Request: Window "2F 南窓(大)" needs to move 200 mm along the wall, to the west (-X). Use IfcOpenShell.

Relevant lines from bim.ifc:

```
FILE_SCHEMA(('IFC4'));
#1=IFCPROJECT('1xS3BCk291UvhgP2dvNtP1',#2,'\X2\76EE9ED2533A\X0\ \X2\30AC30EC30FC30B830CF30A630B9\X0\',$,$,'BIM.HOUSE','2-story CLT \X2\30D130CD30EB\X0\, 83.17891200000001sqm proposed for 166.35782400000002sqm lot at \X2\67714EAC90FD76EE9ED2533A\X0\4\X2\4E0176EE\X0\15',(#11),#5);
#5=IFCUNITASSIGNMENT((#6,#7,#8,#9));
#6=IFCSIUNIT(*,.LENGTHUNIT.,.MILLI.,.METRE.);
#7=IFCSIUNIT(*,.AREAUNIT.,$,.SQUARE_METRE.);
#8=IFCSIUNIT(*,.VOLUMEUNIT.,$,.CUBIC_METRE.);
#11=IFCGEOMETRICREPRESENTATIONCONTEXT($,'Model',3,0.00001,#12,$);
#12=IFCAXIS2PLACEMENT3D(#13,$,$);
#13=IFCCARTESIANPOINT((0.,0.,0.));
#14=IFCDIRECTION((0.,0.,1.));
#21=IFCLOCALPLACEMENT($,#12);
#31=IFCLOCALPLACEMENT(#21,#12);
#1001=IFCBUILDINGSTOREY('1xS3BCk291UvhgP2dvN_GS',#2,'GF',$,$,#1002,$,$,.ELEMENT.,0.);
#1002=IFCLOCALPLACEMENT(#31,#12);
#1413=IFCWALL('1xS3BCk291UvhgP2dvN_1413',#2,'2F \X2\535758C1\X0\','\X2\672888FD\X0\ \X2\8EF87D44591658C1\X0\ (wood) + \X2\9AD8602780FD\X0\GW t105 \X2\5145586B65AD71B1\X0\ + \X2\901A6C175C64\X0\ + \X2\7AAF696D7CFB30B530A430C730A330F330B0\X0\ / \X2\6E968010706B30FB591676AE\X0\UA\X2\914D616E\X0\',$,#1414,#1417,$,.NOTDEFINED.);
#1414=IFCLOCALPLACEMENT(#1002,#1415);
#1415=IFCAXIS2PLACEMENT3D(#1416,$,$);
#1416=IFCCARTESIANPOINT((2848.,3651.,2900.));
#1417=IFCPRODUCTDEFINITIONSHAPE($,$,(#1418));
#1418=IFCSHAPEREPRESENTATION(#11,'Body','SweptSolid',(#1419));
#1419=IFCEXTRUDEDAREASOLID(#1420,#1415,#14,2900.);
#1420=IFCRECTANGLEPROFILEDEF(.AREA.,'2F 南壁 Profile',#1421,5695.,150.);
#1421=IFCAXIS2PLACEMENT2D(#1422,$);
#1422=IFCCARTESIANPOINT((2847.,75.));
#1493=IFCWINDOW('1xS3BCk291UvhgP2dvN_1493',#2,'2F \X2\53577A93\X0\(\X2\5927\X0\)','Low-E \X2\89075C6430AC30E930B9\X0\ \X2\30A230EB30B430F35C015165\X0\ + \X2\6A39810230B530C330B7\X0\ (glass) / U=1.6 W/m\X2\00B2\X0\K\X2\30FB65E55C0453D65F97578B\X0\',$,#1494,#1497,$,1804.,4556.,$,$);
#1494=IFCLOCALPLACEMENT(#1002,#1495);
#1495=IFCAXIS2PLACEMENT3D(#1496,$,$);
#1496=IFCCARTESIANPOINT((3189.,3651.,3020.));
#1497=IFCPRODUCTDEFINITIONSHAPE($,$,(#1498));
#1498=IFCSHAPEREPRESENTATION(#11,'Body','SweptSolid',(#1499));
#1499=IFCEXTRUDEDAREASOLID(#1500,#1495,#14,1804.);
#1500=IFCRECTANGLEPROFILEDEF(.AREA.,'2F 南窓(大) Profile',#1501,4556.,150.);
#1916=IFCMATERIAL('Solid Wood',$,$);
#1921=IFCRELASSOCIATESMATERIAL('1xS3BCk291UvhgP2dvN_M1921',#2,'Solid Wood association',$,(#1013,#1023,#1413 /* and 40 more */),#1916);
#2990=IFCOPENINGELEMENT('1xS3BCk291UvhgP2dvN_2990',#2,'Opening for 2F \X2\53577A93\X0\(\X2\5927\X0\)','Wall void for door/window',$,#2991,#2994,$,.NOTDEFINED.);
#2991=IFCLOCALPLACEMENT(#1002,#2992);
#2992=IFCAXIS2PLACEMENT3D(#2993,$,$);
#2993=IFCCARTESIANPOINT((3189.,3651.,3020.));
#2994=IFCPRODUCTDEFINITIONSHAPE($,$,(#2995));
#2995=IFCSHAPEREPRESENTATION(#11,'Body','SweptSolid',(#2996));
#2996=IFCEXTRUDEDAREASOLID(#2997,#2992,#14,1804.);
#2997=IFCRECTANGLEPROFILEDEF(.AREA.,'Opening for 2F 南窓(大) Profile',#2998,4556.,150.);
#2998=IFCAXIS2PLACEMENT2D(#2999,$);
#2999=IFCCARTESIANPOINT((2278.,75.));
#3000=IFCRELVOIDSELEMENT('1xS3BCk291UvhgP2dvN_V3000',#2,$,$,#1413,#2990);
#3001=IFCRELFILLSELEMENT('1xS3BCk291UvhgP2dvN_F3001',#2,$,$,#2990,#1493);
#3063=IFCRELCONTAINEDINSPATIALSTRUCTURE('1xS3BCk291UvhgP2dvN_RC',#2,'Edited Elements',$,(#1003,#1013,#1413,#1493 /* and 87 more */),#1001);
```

```python
import ifcopenshell
import ifcopenshell.api.geometry
import ifcopenshell.util.placement
import ifcopenshell.util.unit

model = ifcopenshell.open("bim.ifc")
unit_scale = ifcopenshell.util.unit.calculate_unit_scale(model)

window = model.by_guid("1xS3BCk291UvhgP2dvN_1493")
opening = window.FillsVoids[0].RelatingOpeningElement
wall = opening.VoidsElements[0].RelatingBuildingElement

wall_matrix = ifcopenshell.util.placement.get_local_placement(wall.ObjectPlacement)
shift = wall_matrix[:3, 0] * -0.2 / unit_scale
before = ifcopenshell.util.placement.get_local_placement(window.ObjectPlacement)[:3, 3].copy()

# The window is not placed relative to its opening, so move both.
for product in (opening, window):
    matrix = ifcopenshell.util.placement.get_local_placement(product.ObjectPlacement)
    matrix[:3, 3] += shift
    ifcopenshell.api.geometry.edit_object_placement(model, product=product, matrix=matrix, is_si=False)

after = ifcopenshell.util.placement.get_local_placement(window.ObjectPlacement)[:3, 3]
print("window moved by", (after - before).round(3) + 0.0)

model.write("bim_edited.ifc")
```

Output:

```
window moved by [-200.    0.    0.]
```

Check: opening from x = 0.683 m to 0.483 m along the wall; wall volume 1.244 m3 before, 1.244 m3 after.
